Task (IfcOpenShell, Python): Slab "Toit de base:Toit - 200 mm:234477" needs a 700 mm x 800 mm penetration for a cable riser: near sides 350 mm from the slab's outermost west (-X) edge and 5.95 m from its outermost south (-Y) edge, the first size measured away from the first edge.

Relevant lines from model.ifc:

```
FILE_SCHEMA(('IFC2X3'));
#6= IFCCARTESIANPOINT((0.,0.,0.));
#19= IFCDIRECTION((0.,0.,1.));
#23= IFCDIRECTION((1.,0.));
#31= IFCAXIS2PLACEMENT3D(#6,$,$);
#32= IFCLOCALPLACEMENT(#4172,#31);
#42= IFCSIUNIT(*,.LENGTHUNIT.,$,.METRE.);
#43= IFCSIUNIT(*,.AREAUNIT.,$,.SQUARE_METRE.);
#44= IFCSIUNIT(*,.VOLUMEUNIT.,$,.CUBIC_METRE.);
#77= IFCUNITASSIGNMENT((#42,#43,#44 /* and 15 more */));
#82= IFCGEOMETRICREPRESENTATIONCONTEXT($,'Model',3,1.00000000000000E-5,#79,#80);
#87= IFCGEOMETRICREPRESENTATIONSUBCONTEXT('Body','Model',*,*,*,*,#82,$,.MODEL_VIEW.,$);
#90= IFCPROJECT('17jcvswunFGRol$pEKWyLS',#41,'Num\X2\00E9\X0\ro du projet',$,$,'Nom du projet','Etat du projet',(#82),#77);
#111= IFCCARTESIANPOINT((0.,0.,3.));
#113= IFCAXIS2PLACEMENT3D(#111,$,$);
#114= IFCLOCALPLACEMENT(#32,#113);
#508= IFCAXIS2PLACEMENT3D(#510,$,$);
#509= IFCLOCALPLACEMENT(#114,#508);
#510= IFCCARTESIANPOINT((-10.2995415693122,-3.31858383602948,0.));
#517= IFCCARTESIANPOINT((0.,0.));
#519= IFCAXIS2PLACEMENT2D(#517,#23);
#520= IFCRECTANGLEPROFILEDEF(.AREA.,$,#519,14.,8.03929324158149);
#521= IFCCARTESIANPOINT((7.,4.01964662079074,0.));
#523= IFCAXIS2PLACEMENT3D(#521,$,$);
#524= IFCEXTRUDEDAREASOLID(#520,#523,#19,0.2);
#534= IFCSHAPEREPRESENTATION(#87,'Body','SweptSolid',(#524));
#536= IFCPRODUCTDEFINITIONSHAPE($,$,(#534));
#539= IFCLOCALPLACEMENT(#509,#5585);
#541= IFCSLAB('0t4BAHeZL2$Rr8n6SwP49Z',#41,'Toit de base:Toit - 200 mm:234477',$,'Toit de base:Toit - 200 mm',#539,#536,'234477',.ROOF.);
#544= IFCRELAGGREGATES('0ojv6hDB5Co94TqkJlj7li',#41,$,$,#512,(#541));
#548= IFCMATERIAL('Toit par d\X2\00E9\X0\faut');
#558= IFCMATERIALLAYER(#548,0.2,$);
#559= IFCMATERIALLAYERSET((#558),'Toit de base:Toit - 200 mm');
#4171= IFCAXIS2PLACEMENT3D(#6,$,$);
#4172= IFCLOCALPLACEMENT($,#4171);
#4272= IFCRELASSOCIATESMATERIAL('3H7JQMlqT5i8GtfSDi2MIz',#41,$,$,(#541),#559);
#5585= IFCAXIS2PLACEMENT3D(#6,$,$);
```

```python
import numpy as np
import ifcopenshell
import ifcopenshell.api.feature
import ifcopenshell.api.geometry
import ifcopenshell.api.root
import ifcopenshell.geom
import ifcopenshell.util.placement
import ifcopenshell.util.representation
import ifcopenshell.util.shape
import ifcopenshell.util.unit

model = ifcopenshell.open("model.ifc")
unit_scale = ifcopenshell.util.unit.calculate_unit_scale(model)
settings = ifcopenshell.geom.settings()


def volume(element):
    """Net volume in cubic metres, openings subtracted."""
    shape = ifcopenshell.geom.create_shape(settings, element)
    return ifcopenshell.util.shape.get_volume(shape.geometry)


slab = model.by_id(541)
before = volume(slab)

# Extent in the slab's own axes, in metres. The edges named are its -X and -Y sides.
slab_shape = ifcopenshell.geom.create_shape(settings, slab)
vertices = ifcopenshell.util.shape.get_vertices(slab_shape.geometry)
x_min, y_min, bottom = vertices.min(axis=0)
top = vertices[:, 2].max()

opening = ifcopenshell.api.root.create_entity(model, ifc_class="IfcOpeningElement", name="Cable riser opening")
context = ifcopenshell.util.representation.get_context(model, "Model", "Body", "MODEL_VIEW")
width, depth = 0.7, 0.8
outline = [(0.0, 0.0), (width, 0.0), (width, depth), (0.0, depth), (0.0, 0.0)]
# Overshoot both faces by 50 mm so the cut is clean.
shape = ifcopenshell.api.geometry.add_slab_representation(
    model, context=context, depth=top - bottom + 0.1, polyline=outline
)
ifcopenshell.api.geometry.assign_representation(model, product=opening, representation=shape)

matrix = ifcopenshell.util.placement.get_local_placement(slab.ObjectPlacement)
matrix[:, 3] = matrix @ np.append(np.array([x_min + 0.35, y_min + 5.95, bottom - 0.05]) / unit_scale, 1.0)
ifcopenshell.api.geometry.edit_object_placement(model, product=opening, matrix=matrix, is_si=False)
ifcopenshell.api.feature.add_feature(model, feature=opening, element=slab)

after = volume(slab)

print(f"slab volume {before:.3f} -> {after:.3f} m3")

model.write("model_v2.ifc")
```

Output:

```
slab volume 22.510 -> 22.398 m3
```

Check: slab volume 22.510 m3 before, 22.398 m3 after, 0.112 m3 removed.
